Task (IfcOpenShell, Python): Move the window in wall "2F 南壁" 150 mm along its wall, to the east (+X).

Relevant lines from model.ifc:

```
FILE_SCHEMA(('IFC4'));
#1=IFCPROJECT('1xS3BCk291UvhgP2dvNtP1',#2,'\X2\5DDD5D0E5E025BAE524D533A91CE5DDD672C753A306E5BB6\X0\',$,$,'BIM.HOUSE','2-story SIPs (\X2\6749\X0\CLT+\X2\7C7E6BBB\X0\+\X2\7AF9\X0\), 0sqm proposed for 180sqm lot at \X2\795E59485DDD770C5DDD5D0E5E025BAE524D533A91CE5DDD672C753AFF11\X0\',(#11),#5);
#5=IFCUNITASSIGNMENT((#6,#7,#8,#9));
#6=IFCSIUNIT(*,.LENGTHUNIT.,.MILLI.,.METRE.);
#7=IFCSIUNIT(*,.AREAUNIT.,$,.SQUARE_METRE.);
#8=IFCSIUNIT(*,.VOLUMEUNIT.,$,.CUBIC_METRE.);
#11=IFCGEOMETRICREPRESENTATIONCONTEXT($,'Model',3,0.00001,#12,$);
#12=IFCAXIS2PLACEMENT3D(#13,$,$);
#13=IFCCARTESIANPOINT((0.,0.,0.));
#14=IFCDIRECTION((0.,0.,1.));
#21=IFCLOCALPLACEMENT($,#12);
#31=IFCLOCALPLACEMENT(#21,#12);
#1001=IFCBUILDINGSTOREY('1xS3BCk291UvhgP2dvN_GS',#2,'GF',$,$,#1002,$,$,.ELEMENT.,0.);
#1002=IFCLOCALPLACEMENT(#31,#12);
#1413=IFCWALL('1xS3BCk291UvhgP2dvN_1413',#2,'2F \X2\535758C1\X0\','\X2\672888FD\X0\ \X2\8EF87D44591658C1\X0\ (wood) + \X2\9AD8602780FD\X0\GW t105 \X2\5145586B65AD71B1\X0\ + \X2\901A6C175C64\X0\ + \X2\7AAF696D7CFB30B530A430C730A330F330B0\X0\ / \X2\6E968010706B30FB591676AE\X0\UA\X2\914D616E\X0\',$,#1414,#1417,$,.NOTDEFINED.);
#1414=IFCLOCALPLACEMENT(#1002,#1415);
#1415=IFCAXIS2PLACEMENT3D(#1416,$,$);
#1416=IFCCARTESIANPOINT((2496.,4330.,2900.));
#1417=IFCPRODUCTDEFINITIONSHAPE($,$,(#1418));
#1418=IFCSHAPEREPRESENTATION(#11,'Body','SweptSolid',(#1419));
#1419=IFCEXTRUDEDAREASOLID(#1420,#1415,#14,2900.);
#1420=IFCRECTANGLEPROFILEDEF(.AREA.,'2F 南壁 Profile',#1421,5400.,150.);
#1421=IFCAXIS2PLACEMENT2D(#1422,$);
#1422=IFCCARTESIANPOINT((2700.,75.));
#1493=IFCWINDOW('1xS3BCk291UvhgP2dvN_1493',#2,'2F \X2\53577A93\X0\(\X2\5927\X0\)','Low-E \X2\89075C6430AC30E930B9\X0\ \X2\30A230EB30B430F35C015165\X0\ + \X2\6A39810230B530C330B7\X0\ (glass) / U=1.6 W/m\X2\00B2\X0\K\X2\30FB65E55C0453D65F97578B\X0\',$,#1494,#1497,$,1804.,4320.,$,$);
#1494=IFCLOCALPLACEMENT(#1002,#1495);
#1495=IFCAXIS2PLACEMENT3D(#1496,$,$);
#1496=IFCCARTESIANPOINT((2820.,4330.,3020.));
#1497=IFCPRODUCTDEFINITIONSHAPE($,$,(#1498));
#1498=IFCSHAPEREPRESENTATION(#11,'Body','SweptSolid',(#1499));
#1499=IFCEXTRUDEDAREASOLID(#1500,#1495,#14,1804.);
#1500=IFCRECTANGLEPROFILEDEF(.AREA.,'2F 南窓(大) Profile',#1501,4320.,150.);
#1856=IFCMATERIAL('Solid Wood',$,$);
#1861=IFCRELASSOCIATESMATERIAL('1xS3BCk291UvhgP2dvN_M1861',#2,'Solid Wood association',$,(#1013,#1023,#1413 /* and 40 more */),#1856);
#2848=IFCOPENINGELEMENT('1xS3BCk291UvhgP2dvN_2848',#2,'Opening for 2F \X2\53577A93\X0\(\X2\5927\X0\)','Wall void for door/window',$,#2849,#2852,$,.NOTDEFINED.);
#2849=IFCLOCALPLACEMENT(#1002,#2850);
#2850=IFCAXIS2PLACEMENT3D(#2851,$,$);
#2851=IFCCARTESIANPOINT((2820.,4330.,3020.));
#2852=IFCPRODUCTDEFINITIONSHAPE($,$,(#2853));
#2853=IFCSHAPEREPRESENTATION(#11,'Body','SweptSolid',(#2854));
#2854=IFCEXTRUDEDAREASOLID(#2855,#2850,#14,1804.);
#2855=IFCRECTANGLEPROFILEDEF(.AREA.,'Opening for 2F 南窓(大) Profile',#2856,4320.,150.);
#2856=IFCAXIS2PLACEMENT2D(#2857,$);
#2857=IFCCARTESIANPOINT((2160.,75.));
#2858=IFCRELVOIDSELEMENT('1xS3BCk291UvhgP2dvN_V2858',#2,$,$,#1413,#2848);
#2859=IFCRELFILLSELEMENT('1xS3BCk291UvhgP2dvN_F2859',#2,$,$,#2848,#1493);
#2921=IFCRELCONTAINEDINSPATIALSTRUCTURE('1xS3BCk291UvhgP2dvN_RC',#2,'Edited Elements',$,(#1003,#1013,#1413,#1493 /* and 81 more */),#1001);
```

```python
import ifcopenshell
import ifcopenshell.api.geometry
import ifcopenshell.util.placement

model = ifcopenshell.open("model.ifc")

window = model.by_id(1493)
opening = window.FillsVoids[0].RelatingOpeningElement
wall = opening.VoidsElements[0].RelatingBuildingElement

wall_matrix = ifcopenshell.util.placement.get_local_placement(wall.ObjectPlacement)
shift = wall_matrix[:3, 0] * 150.0
before = ifcopenshell.util.placement.get_local_placement(window.ObjectPlacement)[:3, 3].copy()

# The window is not placed relative to its opening, so move both.
for product in (opening, window):
    matrix = ifcopenshell.util.placement.get_local_placement(product.ObjectPlacement)
    matrix[:3, 3] += shift
    ifcopenshell.api.geometry.edit_object_placement(model, product=product, matrix=matrix, is_si=False)

after = ifcopenshell.util.placement.get_local_placement(window.ObjectPlacement)[:3, 3]
print("window moved by", (after - before).round(3) + 0.0)

model.write("model_updated.ifc")
```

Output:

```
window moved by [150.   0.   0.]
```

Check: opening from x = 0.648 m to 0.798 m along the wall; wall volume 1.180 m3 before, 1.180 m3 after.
